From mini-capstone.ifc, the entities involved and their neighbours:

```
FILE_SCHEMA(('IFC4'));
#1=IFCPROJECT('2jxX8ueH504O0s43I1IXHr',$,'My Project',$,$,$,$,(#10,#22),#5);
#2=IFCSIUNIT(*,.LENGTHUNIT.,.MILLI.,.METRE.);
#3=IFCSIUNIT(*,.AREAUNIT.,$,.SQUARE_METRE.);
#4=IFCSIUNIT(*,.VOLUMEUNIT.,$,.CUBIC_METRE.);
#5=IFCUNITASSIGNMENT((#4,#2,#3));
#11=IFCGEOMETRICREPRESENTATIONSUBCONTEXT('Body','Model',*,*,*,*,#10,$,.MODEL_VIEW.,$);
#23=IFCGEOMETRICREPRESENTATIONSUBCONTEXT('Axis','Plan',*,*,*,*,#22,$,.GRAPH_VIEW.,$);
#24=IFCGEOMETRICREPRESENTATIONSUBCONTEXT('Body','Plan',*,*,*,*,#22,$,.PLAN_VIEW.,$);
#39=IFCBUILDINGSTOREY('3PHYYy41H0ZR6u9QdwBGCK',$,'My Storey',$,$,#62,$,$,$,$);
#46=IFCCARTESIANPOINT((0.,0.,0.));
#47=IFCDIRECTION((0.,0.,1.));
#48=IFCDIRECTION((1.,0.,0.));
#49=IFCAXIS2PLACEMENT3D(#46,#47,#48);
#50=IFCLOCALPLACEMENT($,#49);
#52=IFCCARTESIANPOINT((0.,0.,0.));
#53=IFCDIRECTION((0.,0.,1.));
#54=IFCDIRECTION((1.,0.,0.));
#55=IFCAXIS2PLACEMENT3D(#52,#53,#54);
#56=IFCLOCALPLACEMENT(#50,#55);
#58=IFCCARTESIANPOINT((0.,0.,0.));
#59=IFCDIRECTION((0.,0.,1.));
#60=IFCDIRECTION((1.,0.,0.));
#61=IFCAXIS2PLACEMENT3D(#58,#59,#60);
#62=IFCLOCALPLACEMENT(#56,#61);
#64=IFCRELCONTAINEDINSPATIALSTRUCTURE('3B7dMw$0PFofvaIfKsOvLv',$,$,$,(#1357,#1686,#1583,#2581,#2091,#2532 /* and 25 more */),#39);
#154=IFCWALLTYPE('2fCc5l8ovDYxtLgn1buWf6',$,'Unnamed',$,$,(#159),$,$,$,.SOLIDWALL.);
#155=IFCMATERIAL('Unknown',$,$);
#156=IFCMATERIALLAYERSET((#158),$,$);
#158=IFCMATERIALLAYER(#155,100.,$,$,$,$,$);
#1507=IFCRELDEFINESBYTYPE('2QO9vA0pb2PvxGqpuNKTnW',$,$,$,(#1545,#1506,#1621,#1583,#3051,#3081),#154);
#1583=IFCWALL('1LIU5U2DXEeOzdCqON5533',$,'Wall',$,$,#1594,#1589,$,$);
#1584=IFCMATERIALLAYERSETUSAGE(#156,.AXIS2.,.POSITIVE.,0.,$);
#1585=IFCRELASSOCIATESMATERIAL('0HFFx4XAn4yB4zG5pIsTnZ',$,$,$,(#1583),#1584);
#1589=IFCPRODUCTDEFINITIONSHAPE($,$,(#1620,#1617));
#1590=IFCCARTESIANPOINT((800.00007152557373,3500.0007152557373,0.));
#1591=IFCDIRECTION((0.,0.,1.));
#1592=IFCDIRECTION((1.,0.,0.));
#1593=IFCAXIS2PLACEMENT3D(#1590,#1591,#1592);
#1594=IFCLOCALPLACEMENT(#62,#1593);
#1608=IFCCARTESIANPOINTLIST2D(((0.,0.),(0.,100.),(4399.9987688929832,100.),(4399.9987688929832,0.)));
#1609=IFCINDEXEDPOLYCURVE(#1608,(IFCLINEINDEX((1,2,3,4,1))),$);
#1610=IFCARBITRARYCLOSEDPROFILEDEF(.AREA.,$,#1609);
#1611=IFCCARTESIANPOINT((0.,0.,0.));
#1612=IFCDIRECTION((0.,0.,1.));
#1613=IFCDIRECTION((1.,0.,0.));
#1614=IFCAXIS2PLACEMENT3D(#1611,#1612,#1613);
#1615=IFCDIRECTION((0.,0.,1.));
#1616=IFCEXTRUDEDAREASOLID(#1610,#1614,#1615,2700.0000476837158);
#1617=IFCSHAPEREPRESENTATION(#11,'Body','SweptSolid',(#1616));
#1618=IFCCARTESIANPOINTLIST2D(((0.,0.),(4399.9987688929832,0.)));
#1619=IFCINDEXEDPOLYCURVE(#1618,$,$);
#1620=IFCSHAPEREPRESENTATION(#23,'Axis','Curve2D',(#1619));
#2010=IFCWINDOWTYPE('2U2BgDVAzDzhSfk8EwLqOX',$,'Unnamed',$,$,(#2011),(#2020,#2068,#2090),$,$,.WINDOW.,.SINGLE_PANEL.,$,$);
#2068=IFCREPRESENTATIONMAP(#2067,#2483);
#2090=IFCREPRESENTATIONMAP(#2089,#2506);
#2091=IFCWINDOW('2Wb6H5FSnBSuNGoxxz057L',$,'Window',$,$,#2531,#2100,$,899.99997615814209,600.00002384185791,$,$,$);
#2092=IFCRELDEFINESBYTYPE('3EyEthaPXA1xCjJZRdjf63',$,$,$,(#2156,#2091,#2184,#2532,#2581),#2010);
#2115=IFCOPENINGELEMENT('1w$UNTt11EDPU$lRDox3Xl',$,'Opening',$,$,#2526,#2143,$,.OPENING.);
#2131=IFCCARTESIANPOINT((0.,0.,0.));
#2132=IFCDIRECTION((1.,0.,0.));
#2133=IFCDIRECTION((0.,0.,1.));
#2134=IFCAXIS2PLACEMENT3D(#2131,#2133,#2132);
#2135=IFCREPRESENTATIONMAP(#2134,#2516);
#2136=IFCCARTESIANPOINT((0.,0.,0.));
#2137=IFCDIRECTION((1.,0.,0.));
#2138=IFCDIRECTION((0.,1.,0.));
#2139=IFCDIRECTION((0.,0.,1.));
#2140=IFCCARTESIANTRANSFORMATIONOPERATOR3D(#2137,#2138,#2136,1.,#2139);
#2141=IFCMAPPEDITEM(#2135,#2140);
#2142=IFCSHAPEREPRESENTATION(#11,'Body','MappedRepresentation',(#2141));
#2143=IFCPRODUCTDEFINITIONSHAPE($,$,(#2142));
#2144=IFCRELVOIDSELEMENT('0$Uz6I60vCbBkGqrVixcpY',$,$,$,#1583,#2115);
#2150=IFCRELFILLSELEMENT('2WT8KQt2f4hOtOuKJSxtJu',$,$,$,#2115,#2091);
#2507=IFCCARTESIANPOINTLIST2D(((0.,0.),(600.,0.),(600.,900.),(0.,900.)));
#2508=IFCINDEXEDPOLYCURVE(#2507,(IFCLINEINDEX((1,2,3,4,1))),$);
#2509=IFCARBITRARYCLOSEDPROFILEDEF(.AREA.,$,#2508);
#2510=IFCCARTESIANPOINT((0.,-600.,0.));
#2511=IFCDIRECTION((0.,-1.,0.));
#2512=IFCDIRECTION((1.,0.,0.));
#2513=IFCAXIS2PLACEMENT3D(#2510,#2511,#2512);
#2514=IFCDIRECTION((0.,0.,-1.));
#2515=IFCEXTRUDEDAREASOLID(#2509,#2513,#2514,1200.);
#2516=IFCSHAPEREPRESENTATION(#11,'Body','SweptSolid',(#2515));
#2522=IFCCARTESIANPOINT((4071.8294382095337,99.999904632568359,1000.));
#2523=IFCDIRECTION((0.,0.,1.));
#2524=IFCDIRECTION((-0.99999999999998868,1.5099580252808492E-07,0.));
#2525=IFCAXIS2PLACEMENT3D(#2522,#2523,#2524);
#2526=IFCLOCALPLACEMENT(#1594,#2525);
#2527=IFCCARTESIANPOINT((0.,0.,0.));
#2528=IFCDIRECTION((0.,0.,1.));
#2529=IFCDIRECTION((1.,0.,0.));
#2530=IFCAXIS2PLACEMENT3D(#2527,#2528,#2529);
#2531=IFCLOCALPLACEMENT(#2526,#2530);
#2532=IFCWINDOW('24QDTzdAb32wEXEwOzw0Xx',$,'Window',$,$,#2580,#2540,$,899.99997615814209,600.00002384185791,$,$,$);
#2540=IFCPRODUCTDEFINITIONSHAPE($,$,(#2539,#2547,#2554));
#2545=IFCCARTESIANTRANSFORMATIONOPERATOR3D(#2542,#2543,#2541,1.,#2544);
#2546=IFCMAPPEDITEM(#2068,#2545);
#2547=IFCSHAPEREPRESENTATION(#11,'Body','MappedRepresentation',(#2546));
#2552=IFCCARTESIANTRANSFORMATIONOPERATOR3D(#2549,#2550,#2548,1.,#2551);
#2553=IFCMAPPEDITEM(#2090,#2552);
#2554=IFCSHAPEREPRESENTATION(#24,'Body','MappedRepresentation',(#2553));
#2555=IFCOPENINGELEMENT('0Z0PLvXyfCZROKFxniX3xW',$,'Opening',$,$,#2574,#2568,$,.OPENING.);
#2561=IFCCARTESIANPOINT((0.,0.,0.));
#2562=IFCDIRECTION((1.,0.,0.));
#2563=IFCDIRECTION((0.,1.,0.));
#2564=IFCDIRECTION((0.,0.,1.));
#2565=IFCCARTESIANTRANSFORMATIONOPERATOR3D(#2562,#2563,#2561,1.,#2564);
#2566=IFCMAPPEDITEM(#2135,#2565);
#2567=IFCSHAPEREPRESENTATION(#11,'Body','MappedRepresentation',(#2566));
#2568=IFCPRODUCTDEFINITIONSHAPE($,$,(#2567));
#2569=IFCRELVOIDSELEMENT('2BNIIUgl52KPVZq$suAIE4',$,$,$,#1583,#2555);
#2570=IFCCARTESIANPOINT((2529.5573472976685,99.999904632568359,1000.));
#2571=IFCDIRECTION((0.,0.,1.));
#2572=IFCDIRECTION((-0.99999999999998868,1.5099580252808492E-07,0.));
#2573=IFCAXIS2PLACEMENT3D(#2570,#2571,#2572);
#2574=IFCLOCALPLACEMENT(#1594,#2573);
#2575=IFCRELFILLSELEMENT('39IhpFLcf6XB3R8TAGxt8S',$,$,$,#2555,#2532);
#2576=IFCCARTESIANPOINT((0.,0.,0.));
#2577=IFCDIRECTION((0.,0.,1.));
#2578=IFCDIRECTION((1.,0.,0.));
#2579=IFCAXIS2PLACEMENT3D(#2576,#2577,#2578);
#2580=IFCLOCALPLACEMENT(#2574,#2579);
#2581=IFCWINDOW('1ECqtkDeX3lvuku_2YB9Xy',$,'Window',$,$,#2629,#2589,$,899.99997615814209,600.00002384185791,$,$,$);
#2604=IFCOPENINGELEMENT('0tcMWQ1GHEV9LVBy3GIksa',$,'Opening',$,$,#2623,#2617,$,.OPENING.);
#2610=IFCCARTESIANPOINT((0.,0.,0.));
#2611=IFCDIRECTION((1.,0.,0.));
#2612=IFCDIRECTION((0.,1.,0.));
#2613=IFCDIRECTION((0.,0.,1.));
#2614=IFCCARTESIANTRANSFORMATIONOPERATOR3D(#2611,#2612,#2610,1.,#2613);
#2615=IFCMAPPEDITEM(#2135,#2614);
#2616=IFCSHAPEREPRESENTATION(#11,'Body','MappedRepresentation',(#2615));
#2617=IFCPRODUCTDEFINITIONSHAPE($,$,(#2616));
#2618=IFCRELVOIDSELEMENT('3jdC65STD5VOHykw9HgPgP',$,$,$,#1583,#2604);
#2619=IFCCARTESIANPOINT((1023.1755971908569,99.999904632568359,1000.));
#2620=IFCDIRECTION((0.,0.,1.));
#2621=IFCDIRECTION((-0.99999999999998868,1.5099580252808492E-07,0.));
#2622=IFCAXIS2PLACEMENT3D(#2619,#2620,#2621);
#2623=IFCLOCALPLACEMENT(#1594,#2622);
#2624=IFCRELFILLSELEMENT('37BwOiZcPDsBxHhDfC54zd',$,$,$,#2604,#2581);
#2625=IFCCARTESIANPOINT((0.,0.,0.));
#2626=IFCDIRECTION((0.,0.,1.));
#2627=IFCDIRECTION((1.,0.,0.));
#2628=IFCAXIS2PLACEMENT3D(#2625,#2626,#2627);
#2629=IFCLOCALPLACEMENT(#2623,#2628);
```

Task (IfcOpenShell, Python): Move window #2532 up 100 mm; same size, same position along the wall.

```python
import numpy as np
import ifcopenshell
import ifcopenshell.api.geometry
import ifcopenshell.util.placement
import ifcopenshell.util.unit

model = ifcopenshell.open("mini-capstone.ifc")
unit_scale = ifcopenshell.util.unit.calculate_unit_scale(model)

window = model.by_id(2532)
opening = window.FillsVoids[0].RelatingOpeningElement
dz = 0.1 / unit_scale

shift = np.array([0.0, 0.0, dz])
# The window is placed relative to its opening, so it follows when the opening moves.
matrix = ifcopenshell.util.placement.get_local_placement(opening.ObjectPlacement)
matrix[:3, 3] += shift
ifcopenshell.api.geometry.edit_object_placement(
    model, product=opening, matrix=matrix, is_si=False, should_transform_children=True
)

print(f"moved by {dz * unit_scale:+.3f} m")

model.write("mini-capstone-out.ifc")
```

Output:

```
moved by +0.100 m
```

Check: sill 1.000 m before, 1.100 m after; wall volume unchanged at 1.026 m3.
